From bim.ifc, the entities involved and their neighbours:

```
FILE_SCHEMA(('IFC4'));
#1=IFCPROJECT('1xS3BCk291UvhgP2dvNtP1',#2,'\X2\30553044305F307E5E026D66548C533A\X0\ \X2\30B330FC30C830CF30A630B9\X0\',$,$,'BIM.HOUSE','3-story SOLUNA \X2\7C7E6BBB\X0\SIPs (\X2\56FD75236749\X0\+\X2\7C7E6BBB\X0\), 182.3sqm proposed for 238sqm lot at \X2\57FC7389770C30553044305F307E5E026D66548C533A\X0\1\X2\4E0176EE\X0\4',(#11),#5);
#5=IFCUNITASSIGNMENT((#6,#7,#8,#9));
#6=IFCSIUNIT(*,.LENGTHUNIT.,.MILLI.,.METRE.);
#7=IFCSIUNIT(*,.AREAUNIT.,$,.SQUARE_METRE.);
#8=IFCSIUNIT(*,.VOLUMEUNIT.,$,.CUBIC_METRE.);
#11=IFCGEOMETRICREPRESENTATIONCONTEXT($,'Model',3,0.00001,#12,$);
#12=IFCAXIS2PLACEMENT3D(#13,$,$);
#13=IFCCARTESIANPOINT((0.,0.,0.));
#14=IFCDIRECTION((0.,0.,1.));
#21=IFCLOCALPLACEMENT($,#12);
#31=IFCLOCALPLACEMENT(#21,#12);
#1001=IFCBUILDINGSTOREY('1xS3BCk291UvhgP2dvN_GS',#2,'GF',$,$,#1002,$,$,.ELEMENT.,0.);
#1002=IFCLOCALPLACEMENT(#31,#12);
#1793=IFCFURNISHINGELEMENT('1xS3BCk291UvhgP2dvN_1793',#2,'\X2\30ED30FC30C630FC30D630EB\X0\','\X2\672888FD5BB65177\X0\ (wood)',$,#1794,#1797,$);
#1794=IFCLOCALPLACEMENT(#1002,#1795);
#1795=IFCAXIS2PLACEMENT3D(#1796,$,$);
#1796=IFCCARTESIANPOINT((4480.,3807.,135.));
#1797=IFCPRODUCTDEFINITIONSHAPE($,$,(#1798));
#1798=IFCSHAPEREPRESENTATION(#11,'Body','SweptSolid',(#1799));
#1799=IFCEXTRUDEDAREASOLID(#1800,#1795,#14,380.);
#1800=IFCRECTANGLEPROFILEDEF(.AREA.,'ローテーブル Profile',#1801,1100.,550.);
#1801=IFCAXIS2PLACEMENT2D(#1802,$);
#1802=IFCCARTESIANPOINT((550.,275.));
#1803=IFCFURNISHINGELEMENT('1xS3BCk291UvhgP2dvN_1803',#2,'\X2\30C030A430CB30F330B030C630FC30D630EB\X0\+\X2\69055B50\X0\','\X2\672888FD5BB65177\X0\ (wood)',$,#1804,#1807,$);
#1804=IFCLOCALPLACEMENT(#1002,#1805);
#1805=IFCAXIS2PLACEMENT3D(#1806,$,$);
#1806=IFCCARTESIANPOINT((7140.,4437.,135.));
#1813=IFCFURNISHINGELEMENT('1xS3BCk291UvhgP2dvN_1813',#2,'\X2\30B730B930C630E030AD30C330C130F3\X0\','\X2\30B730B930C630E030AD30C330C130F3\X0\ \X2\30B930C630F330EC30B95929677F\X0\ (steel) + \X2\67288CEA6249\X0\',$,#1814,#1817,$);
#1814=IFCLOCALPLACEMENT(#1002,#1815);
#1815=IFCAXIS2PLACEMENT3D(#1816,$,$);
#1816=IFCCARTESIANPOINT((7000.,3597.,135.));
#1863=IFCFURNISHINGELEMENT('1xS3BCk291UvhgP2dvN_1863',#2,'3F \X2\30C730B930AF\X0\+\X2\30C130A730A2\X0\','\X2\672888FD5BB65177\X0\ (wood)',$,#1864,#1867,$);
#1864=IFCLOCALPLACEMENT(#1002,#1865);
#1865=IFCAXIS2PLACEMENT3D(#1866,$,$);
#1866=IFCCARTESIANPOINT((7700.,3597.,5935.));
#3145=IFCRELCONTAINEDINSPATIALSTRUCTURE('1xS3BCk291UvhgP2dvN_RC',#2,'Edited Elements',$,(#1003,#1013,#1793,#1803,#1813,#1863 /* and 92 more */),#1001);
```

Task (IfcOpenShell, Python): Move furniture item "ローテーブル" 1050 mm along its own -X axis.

```python
import ifcopenshell
import ifcopenshell.api.geometry
import ifcopenshell.util.placement
import ifcopenshell.util.unit

model = ifcopenshell.open("bim.ifc")
unit_scale = ifcopenshell.util.unit.calculate_unit_scale(model)

item = model.by_id(1793)
matrix = ifcopenshell.util.placement.get_local_placement(item.ObjectPlacement)
matrix[:3, 3] -= matrix[:3, 0] * 1.05 / unit_scale
ifcopenshell.api.geometry.edit_object_placement(model, product=item, matrix=matrix, is_si=False)

print(ifcopenshell.util.placement.get_local_placement(item.ObjectPlacement).round(3) + 0.0)

model.write("bim_updated.ifc")
```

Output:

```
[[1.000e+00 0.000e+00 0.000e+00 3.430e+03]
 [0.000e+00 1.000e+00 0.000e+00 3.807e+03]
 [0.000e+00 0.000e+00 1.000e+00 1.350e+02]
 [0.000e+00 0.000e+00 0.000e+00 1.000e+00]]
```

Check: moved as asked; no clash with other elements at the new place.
